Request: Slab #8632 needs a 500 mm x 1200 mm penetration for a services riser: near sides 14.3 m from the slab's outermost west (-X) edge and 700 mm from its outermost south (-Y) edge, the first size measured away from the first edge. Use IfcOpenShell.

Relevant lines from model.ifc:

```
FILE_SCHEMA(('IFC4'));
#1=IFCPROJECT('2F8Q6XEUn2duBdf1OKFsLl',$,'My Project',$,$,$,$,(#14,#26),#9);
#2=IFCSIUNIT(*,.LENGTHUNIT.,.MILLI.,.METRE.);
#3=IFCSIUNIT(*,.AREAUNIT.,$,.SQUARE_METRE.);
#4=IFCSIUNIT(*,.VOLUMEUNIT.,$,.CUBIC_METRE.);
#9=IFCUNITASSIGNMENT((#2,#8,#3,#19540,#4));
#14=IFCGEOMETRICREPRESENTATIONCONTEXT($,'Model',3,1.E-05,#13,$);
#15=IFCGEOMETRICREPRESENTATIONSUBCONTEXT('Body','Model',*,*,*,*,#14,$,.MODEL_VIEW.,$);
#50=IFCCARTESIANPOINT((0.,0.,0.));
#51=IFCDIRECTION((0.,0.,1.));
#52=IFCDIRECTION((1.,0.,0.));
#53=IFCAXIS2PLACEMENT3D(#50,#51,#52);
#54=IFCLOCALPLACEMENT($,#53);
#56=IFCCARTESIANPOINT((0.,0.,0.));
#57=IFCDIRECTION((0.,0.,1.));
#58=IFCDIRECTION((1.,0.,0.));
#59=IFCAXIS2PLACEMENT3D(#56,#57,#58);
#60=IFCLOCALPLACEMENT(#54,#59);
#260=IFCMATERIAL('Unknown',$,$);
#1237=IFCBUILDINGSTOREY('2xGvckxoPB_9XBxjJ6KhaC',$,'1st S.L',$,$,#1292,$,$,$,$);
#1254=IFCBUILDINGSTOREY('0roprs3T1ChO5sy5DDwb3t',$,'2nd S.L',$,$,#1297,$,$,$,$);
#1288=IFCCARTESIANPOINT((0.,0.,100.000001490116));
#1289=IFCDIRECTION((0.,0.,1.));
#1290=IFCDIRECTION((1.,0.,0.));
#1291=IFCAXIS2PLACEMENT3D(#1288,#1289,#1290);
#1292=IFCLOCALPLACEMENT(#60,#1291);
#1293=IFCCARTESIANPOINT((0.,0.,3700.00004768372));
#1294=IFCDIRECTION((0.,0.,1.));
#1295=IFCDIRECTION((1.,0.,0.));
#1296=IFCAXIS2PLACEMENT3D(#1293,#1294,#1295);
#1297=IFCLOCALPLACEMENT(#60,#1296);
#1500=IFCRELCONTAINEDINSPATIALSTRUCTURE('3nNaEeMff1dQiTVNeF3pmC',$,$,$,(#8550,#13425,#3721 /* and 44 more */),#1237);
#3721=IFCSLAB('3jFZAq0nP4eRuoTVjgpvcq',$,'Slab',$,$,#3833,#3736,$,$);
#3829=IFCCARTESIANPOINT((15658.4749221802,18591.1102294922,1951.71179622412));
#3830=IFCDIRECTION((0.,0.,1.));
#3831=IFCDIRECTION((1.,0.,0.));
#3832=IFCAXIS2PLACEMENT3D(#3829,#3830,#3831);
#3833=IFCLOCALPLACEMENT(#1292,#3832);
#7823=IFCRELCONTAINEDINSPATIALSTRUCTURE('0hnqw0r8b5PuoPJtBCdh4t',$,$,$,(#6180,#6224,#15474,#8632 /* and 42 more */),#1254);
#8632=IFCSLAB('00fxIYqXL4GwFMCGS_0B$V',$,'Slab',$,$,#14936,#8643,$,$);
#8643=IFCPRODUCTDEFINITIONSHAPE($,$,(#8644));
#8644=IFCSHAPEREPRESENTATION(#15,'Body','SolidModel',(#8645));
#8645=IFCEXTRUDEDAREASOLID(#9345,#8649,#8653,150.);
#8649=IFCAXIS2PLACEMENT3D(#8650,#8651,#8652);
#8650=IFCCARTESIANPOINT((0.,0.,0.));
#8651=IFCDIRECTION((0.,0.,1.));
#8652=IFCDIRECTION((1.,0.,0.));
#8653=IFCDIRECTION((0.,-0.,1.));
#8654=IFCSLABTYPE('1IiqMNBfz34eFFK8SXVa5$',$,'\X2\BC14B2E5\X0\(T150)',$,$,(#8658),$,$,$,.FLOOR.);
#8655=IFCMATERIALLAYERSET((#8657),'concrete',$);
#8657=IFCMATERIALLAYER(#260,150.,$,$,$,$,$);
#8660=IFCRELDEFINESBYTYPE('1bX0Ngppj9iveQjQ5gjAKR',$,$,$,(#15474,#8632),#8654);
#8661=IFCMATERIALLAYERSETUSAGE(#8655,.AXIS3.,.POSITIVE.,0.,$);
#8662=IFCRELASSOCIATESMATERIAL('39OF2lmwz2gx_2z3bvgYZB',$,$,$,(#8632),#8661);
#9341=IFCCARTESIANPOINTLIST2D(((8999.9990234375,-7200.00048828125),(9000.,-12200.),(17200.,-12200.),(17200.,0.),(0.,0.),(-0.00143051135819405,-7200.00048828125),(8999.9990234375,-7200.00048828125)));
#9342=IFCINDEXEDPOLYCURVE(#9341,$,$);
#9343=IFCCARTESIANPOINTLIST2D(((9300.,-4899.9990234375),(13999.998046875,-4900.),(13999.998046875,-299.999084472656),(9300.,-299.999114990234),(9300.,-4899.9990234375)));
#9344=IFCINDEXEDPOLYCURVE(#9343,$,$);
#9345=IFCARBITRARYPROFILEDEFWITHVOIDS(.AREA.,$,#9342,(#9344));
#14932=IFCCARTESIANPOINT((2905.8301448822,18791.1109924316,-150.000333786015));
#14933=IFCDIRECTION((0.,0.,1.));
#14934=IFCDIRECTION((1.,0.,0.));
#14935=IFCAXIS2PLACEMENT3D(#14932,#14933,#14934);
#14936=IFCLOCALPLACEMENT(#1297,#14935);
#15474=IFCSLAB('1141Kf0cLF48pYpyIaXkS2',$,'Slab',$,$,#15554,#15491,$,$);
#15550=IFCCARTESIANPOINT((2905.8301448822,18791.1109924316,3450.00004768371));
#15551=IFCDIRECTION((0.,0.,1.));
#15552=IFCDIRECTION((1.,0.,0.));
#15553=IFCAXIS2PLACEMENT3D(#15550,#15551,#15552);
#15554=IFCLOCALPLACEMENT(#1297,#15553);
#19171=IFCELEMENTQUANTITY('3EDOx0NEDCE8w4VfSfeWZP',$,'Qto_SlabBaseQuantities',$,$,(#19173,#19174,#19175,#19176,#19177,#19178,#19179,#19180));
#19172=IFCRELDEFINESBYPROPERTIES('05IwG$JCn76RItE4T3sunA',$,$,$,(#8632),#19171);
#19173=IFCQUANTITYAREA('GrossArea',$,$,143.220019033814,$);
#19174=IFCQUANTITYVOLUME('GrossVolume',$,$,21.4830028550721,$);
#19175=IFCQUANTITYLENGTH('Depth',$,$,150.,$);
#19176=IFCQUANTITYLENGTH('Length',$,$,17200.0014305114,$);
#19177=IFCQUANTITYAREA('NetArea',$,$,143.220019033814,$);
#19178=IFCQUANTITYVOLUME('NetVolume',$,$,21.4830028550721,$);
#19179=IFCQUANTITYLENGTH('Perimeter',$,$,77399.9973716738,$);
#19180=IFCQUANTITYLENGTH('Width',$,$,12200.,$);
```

```python
import numpy as np
import ifcopenshell
import ifcopenshell.api.feature
import ifcopenshell.api.geometry
import ifcopenshell.api.pset
import ifcopenshell.api.root
import ifcopenshell.geom
import ifcopenshell.util.element
import ifcopenshell.util.placement
import ifcopenshell.util.representation
import ifcopenshell.util.shape
import ifcopenshell.util.unit

model = ifcopenshell.open("model.ifc")
unit_scale = ifcopenshell.util.unit.calculate_unit_scale(model)
area_scale = ifcopenshell.util.unit.calculate_unit_scale(model, "AREAUNIT")
volume_scale = ifcopenshell.util.unit.calculate_unit_scale(model, "VOLUMEUNIT")
settings = ifcopenshell.geom.settings()


def volume(element):
    """Net volume in cubic metres, openings subtracted."""
    shape = ifcopenshell.geom.create_shape(settings, element)
    return ifcopenshell.util.shape.get_volume(shape.geometry)


slab = model.by_guid("00fxIYqXL4GwFMCGS_0B$V")
before = volume(slab)

# Extent in the slab's own axes, in metres. The edges named are its -X and -Y sides.
slab_shape = ifcopenshell.geom.create_shape(settings, slab)
vertices = ifcopenshell.util.shape.get_vertices(slab_shape.geometry)
x_min, y_min, bottom = vertices.min(axis=0)
top = vertices[:, 2].max()

opening = ifcopenshell.api.root.create_entity(model, ifc_class="IfcOpeningElement", name="Services riser opening", predefined_type="OPENING")
context = ifcopenshell.util.representation.get_context(model, "Model", "Body", "MODEL_VIEW")
width, depth = 0.5, 1.2
outline = [(0.0, 0.0), (width, 0.0), (width, depth), (0.0, depth), (0.0, 0.0)]
# Overshoot both faces by 50 mm so the cut is clean.
shape = ifcopenshell.api.geometry.add_slab_representation(
    model, context=context, depth=top - bottom + 0.1, polyline=outline
)
ifcopenshell.api.geometry.assign_representation(model, product=opening, representation=shape)

matrix = ifcopenshell.util.placement.get_local_placement(slab.ObjectPlacement)
matrix[:, 3] = matrix @ np.append(np.array([x_min + 14.3, y_min + 0.7, bottom - 0.05]) / unit_scale, 1.0)
ifcopenshell.api.geometry.edit_object_placement(model, product=opening, matrix=matrix, is_si=False)
ifcopenshell.api.feature.add_feature(model, feature=opening, element=slab)

after = volume(slab)

# Update the slab's stored quantities.
qto = model.by_id(ifcopenshell.util.element.get_pset(slab, "Qto_SlabBaseQuantities", should_inherit=False)["id"])
ifcopenshell.api.pset.edit_qto(model, qto=qto, properties={
    "NetArea": after / (top - bottom) / area_scale,
    "NetVolume": after / volume_scale,
})

print(f"slab volume {before:.3f} -> {after:.3f} m3")

model.write("model_edited.ifc")
```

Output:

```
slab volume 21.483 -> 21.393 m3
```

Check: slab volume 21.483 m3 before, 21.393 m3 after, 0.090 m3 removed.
